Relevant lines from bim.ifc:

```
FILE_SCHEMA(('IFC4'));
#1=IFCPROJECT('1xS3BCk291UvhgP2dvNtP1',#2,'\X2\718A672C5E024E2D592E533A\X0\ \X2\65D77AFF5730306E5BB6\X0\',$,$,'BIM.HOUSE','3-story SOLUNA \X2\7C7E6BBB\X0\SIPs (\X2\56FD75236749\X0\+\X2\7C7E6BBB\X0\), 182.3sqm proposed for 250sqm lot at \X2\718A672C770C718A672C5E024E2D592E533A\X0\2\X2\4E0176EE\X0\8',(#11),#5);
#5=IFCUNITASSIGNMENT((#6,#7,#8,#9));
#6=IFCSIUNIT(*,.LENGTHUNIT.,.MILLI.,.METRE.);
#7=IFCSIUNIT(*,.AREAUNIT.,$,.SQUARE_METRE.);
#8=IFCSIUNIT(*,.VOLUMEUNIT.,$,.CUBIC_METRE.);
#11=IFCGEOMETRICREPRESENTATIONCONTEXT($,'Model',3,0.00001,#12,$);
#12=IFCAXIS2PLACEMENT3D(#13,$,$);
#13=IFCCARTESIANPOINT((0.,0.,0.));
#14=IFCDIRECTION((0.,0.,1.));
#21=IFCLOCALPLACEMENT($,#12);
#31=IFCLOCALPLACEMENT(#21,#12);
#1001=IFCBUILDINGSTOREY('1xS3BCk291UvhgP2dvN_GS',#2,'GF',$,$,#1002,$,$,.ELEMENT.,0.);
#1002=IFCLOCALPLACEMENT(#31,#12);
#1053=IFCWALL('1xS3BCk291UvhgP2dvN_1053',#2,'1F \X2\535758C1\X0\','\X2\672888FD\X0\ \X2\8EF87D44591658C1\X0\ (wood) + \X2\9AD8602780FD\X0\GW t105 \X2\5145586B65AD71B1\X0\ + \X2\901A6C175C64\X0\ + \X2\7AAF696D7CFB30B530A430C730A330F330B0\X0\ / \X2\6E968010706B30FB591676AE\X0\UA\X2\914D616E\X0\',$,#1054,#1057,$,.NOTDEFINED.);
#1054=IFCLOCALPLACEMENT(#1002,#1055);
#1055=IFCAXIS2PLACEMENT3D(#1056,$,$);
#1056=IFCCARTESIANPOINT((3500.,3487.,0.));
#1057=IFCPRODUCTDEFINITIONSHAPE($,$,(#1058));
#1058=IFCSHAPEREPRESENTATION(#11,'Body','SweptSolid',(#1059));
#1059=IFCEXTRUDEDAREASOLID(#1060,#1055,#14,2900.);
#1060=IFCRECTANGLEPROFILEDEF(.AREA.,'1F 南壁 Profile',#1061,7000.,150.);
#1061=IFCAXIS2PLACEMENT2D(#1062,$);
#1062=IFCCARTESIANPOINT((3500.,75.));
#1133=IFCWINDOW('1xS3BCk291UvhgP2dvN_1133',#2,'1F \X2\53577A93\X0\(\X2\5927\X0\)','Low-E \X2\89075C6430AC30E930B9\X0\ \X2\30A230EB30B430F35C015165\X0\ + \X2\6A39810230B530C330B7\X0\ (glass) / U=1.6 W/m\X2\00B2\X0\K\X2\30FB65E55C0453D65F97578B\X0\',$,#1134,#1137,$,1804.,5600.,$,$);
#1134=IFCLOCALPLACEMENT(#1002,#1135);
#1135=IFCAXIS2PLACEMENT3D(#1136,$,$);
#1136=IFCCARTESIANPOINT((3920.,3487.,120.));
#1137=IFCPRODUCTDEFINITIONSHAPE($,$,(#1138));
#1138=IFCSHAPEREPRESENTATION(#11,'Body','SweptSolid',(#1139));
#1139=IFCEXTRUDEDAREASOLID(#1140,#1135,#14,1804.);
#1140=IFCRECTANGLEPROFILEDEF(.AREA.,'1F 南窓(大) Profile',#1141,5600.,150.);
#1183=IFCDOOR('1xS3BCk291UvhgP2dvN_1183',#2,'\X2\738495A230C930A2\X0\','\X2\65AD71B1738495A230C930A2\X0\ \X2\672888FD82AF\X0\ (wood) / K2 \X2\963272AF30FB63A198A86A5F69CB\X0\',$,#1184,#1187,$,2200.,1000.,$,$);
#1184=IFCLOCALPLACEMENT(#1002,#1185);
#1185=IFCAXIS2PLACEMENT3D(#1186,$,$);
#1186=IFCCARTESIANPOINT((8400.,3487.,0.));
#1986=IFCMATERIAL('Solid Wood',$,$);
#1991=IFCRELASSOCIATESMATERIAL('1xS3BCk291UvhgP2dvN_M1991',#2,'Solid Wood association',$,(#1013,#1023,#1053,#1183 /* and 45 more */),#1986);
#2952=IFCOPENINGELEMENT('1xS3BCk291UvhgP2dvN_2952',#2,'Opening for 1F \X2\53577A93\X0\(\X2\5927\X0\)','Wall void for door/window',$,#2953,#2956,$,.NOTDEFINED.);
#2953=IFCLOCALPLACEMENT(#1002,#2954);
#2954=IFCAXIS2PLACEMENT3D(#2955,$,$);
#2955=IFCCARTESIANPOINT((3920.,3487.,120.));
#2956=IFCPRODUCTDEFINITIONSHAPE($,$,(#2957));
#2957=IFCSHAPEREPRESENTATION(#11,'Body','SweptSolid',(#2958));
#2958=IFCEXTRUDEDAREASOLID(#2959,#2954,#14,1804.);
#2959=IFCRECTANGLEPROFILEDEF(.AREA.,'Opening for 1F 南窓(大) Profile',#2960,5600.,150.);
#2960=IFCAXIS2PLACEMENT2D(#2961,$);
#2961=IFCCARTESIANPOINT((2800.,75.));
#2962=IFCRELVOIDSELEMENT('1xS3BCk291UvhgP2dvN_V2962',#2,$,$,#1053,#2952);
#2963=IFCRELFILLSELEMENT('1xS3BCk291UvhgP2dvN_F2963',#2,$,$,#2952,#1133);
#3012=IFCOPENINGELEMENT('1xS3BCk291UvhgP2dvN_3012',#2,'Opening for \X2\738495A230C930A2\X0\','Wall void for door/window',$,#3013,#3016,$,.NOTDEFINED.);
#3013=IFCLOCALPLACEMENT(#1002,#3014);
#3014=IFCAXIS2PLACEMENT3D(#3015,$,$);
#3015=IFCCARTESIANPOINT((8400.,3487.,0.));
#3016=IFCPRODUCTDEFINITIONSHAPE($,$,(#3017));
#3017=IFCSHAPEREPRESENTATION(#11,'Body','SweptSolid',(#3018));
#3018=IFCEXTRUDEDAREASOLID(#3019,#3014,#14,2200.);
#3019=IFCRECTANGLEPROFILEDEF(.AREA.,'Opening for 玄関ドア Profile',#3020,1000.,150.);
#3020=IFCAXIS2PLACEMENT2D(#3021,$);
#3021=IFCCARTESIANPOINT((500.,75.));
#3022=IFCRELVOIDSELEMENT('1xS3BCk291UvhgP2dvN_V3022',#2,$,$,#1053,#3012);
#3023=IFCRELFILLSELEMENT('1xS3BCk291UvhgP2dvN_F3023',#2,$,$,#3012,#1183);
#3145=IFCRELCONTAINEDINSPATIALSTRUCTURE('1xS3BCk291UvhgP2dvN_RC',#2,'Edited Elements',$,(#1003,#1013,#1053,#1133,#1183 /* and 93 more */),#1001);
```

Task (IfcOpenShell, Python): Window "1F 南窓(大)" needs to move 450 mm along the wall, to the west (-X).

```python
import ifcopenshell
import ifcopenshell.api.geometry
import ifcopenshell.util.placement
import ifcopenshell.util.unit

model = ifcopenshell.open("bim.ifc")
unit_scale = ifcopenshell.util.unit.calculate_unit_scale(model)

window = model.by_guid("1xS3BCk291UvhgP2dvN_1133")
opening = window.FillsVoids[0].RelatingOpeningElement
wall = opening.VoidsElements[0].RelatingBuildingElement

wall_matrix = ifcopenshell.util.placement.get_local_placement(wall.ObjectPlacement)
shift = wall_matrix[:3, 0] * -0.45 / unit_scale
before = ifcopenshell.util.placement.get_local_placement(window.ObjectPlacement)[:3, 3].copy()

# The window is not placed relative to its opening, so move both.
for product in (opening, window):
    matrix = ifcopenshell.util.placement.get_local_placement(product.ObjectPlacement)
    matrix[:3, 3] += shift
    ifcopenshell.api.geometry.edit_object_placement(model, product=product, matrix=matrix, is_si=False)

after = ifcopenshell.util.placement.get_local_placement(window.ObjectPlacement)[:3, 3]
print("window moved by", (after - before).round(3) + 0.0)

model.write("bim_v2.ifc")
```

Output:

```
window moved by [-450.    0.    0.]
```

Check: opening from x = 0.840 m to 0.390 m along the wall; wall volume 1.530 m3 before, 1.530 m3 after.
